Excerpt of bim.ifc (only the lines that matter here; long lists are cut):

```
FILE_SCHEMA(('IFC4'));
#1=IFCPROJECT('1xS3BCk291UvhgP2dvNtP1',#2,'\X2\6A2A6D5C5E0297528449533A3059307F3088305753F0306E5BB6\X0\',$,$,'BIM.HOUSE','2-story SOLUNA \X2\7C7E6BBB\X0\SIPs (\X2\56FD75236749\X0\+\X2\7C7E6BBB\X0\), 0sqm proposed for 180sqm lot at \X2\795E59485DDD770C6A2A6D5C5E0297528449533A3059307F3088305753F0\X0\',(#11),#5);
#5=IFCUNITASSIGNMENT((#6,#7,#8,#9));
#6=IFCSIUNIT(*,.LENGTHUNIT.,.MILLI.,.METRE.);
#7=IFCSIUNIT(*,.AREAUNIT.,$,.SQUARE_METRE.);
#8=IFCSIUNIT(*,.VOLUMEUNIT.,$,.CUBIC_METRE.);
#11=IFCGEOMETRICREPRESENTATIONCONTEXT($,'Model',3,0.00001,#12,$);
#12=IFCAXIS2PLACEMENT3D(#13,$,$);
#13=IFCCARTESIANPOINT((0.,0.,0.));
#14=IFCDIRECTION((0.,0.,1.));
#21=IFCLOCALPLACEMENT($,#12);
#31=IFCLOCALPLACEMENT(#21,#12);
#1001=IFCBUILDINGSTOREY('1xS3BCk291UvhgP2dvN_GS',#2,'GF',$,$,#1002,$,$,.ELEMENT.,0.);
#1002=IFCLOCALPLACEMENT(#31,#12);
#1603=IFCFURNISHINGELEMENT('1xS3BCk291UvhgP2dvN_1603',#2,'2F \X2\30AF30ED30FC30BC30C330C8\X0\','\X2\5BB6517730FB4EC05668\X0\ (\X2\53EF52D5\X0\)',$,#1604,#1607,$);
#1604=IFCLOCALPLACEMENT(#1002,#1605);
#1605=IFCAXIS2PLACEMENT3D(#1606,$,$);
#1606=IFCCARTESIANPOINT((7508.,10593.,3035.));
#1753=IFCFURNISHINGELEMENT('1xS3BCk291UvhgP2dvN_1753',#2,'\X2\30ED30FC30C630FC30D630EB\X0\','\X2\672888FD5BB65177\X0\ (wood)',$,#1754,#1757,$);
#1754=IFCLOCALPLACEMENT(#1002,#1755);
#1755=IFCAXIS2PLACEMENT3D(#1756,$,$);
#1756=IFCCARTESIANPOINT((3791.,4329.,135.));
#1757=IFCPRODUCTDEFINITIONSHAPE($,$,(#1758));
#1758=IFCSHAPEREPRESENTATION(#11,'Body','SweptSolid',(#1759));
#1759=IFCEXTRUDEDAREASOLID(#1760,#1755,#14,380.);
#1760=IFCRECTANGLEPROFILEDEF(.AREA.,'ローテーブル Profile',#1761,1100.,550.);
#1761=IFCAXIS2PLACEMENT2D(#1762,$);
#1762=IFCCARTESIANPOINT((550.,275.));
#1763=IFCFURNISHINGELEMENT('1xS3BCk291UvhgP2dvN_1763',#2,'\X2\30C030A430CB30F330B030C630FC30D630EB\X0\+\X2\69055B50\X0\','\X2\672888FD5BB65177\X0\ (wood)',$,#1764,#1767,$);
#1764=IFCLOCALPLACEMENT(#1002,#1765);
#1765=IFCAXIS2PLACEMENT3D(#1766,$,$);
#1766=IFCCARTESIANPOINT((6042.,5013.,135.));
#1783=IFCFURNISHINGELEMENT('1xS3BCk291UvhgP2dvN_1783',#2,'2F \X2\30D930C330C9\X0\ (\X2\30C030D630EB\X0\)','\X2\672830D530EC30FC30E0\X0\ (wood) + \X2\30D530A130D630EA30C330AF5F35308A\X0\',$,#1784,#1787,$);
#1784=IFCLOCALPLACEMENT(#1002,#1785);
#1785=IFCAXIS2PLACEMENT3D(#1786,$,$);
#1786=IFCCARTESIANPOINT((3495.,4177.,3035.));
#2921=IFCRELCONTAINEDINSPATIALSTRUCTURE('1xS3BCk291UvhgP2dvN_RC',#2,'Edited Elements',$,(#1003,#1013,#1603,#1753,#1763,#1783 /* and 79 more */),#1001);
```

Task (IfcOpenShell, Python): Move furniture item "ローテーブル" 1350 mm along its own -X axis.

```python
import ifcopenshell
import ifcopenshell.api.geometry
import ifcopenshell.util.placement
import ifcopenshell.util.unit

model = ifcopenshell.open("bim.ifc")
unit_scale = ifcopenshell.util.unit.calculate_unit_scale(model)

item = model.by_id(1753)
matrix = ifcopenshell.util.placement.get_local_placement(item.ObjectPlacement)
matrix[:3, 3] -= matrix[:3, 0] * 1.35 / unit_scale
ifcopenshell.api.geometry.edit_object_placement(model, product=item, matrix=matrix, is_si=False)

print(ifcopenshell.util.placement.get_local_placement(item.ObjectPlacement).round(3) + 0.0)

model.write("bim-out.ifc")
```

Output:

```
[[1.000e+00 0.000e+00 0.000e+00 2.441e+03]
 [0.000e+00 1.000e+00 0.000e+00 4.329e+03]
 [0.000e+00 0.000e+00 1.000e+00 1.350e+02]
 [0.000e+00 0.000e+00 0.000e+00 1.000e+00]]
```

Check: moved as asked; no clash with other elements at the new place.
